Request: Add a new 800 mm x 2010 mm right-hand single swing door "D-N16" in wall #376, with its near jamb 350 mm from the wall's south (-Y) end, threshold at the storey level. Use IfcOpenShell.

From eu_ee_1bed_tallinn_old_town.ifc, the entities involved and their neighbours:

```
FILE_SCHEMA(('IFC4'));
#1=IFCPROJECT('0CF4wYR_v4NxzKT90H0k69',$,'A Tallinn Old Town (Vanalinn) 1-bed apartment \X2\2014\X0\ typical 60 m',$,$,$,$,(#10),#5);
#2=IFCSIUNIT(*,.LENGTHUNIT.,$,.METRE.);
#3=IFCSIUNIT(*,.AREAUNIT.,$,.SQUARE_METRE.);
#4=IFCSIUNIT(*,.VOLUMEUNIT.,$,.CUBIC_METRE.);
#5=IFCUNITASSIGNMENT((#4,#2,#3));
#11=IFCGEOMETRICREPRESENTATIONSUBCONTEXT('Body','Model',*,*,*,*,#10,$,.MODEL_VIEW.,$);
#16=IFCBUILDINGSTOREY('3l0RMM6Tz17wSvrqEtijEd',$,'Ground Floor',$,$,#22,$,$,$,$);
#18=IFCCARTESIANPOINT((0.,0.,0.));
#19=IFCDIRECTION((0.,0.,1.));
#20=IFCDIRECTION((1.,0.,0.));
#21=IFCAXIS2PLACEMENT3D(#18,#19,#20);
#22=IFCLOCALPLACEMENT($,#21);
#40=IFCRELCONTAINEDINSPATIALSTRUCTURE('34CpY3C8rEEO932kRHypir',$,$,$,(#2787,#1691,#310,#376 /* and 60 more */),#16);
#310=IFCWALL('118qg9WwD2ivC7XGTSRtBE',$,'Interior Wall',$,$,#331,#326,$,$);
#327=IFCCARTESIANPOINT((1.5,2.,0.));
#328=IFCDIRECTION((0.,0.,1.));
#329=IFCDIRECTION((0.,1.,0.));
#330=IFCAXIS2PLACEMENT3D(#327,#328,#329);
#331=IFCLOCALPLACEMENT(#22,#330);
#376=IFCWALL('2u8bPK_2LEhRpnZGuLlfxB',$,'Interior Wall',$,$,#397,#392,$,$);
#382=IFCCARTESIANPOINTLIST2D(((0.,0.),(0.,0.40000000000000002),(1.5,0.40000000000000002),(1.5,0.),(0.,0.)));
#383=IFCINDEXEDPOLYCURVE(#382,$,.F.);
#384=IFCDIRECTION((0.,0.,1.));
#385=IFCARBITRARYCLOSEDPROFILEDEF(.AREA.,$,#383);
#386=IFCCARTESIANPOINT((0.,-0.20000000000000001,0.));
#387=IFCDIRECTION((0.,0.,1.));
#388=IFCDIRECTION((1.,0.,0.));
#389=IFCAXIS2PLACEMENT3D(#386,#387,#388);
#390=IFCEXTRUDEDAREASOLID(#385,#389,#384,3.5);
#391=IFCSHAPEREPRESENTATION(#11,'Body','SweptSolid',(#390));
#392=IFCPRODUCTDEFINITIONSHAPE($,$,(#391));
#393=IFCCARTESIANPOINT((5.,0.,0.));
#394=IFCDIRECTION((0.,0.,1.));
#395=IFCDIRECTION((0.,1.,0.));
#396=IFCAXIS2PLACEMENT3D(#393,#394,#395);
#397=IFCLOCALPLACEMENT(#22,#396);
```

```python
import numpy as np
import ifcopenshell
import ifcopenshell.api.feature
import ifcopenshell.api.geometry
import ifcopenshell.api.root
import ifcopenshell.api.spatial
import ifcopenshell.geom
import ifcopenshell.util.element
import ifcopenshell.util.placement
import ifcopenshell.util.representation
import ifcopenshell.util.shape
import ifcopenshell.util.unit

model = ifcopenshell.open("eu_ee_1bed_tallinn_old_town.ifc")
unit_scale = ifcopenshell.util.unit.calculate_unit_scale(model)
settings = ifcopenshell.geom.settings()


def volume(element):
    """Net volume in cubic metres, openings subtracted."""
    shape = ifcopenshell.geom.create_shape(settings, element)
    return ifcopenshell.util.shape.get_volume(shape.geometry)


wall = model.by_guid("2u8bPK_2LEhRpnZGuLlfxB")
storey = ifcopenshell.util.element.get_container(wall, ifc_class="IfcBuildingStorey")
context = ifcopenshell.util.representation.get_context(model, "Model", "Body", "MODEL_VIEW")
before = volume(wall)

width, height, from_end, sill = 0.8, 2.01, 0.35, 0.0  # metres

# The wall runs along its own X axis, and the end named is its -X end.
wall_shape = ifcopenshell.geom.create_shape(settings, wall)
x, y, z = ifcopenshell.util.shape.get_vertices(wall_shape.geometry).T
start = x.min() + from_end
face, thickness = float(y.min()), float(y.max() - y.min())
wall_matrix = ifcopenshell.util.placement.get_local_placement(wall.ObjectPlacement)
level = ifcopenshell.util.placement.get_local_placement(storey.ObjectPlacement)[2, 3]


def in_wall(x, y):
    """Placement at x, y metres in the wall's axes, at sill height."""
    matrix = wall_matrix.copy()
    matrix[:, 3] = wall_matrix @ np.array([x / unit_scale, y / unit_scale, 0.0, 1.0])
    matrix[2, 3] = level + sill / unit_scale
    return matrix


# Opening: a box that overshoots both wall faces by 50 mm.
opening = ifcopenshell.api.root.create_entity(model, ifc_class="IfcOpeningElement", predefined_type="OPENING")
box = ifcopenshell.api.geometry.add_wall_representation(
    model, context=context, length=width, height=height, thickness=thickness + 0.1
)
ifcopenshell.api.geometry.assign_representation(model, product=opening, representation=box)
ifcopenshell.api.geometry.edit_object_placement(model, product=opening, matrix=in_wall(start, face - 0.05), is_si=False)
ifcopenshell.api.feature.add_feature(model, feature=opening, element=wall)

door = ifcopenshell.api.root.create_entity(model, ifc_class="IfcDoor", name="D-N16", predefined_type="DOOR")
door.OverallWidth, door.OverallHeight = width / unit_scale, height / unit_scale
door.OperationType = "SINGLE_SWING_RIGHT"
body = ifcopenshell.api.geometry.add_door_representation(
    model,
    context=context,
    overall_width=door.OverallWidth,
    overall_height=door.OverallHeight,
    operation_type="SINGLE_SWING_RIGHT",
    lining_properties={"LiningDepth": thickness / unit_scale, "ThresholdDepth": thickness / unit_scale},
)
ifcopenshell.api.geometry.assign_representation(model, product=door, representation=body)
ifcopenshell.api.spatial.assign_container(model, products=[door], relating_structure=storey)
ifcopenshell.api.feature.add_filling(model, opening=opening, element=door)

# The lining spans the wall, so the door starts at the wall face.
ifcopenshell.api.geometry.edit_object_placement(model, product=door, matrix=in_wall(start, face), is_si=False)

after = volume(wall)

print(f"wall volume {before:.3f} -> {after:.3f} m3")

model.write("eu_ee_1bed_tallinn_old_town_v2.ifc")
```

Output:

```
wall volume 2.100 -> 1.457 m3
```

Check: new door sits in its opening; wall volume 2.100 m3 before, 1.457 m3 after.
